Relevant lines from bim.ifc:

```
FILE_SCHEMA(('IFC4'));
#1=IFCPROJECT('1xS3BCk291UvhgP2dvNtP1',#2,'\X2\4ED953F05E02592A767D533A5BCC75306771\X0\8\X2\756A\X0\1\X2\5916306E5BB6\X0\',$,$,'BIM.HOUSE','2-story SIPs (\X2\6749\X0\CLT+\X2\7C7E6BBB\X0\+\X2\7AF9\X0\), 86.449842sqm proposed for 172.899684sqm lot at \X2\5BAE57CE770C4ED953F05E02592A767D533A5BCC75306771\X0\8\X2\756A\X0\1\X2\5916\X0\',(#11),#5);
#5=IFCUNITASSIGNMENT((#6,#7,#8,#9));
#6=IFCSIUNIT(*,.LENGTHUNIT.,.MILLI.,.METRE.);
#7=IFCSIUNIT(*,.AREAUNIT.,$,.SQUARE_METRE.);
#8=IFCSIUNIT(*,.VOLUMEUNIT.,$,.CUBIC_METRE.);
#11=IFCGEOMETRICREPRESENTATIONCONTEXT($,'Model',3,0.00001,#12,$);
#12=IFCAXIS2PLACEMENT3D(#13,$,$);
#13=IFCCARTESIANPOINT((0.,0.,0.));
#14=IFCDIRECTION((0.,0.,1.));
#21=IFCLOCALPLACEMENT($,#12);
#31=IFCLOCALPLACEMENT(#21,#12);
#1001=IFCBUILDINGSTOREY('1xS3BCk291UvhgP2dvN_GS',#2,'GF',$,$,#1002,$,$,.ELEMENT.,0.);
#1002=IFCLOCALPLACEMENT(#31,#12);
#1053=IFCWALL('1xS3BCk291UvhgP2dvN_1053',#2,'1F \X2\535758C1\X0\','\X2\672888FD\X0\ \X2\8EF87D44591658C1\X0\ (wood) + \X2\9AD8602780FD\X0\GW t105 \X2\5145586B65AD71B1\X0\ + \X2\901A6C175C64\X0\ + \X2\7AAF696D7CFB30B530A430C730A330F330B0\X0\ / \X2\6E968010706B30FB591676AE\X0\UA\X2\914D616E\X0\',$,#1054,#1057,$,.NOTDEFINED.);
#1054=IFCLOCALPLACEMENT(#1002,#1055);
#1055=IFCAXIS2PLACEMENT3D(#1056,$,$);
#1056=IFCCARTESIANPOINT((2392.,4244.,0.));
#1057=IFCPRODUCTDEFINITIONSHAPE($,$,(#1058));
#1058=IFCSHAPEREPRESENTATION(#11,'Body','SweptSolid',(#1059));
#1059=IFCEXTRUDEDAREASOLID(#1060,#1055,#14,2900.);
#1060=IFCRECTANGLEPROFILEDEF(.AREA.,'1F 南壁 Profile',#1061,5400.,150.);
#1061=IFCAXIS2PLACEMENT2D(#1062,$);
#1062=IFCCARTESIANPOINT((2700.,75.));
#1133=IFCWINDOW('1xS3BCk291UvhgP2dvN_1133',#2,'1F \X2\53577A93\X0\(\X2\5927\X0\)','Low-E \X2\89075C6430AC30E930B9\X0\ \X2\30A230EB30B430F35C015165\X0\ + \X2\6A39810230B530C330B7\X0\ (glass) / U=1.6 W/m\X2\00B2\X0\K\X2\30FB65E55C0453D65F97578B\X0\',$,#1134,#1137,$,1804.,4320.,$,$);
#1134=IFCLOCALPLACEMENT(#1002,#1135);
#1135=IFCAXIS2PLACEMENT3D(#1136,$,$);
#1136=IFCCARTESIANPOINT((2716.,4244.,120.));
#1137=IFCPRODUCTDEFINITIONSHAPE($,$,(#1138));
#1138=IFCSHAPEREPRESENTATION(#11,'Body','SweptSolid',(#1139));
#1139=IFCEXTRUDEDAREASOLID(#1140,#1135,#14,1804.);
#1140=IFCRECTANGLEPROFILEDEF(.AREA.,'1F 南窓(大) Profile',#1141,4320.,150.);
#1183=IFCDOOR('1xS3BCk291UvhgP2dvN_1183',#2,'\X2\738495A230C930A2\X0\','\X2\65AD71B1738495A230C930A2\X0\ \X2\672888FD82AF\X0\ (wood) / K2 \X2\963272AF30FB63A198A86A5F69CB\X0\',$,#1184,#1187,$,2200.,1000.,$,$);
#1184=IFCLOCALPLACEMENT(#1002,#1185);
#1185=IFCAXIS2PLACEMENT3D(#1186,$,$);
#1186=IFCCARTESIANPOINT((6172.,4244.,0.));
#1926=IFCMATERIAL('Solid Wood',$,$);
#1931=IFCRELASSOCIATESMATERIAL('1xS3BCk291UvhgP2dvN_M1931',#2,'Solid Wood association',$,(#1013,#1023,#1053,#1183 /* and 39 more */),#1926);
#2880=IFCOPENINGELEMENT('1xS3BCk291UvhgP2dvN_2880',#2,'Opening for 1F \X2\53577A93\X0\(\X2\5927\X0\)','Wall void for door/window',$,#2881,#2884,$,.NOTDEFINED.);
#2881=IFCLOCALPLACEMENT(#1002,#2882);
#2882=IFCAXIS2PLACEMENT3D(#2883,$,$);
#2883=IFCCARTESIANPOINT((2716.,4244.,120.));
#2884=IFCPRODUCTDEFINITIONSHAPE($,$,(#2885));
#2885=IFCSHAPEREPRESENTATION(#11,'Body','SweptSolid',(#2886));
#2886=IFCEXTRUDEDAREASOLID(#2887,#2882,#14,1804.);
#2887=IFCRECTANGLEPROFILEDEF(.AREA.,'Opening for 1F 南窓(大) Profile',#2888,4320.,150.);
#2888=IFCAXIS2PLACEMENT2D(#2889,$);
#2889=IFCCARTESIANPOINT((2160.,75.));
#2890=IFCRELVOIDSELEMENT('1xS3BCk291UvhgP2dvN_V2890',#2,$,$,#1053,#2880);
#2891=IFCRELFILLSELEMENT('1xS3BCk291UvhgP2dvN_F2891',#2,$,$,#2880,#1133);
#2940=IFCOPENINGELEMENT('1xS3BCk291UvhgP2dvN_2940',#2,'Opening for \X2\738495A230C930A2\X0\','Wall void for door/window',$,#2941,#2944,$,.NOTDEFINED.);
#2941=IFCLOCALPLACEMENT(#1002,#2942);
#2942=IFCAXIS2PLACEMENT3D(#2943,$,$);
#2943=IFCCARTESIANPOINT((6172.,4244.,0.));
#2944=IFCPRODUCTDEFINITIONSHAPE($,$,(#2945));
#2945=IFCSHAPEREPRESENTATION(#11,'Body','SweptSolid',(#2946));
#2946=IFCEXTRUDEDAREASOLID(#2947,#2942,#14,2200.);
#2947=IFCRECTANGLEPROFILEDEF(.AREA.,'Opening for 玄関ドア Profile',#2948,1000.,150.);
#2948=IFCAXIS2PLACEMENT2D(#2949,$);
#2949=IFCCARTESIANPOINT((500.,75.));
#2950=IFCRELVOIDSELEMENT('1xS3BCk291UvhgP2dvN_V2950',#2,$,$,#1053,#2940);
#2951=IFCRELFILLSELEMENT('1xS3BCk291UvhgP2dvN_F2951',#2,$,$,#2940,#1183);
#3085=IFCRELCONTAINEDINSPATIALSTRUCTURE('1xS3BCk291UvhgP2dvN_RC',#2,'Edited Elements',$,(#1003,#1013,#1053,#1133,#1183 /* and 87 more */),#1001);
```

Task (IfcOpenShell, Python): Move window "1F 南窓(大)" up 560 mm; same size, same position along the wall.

```python
import numpy as np
import ifcopenshell
import ifcopenshell.api.geometry
import ifcopenshell.util.placement
import ifcopenshell.util.unit

model = ifcopenshell.open("bim.ifc")
unit_scale = ifcopenshell.util.unit.calculate_unit_scale(model)

window = model.by_guid("1xS3BCk291UvhgP2dvN_1133")
opening = window.FillsVoids[0].RelatingOpeningElement
dz = 560.0

shift = np.array([0.0, 0.0, dz])
# The window is not placed relative to its opening, so move both.
for product in (opening, window):
    matrix = ifcopenshell.util.placement.get_local_placement(product.ObjectPlacement)
    matrix[:3, 3] += shift
    ifcopenshell.api.geometry.edit_object_placement(model, product=product, matrix=matrix, is_si=False)

print(f"moved by {dz * unit_scale:+.3f} m")

model.write("bim_v2.ifc")
```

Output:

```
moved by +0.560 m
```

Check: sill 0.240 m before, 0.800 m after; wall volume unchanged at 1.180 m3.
